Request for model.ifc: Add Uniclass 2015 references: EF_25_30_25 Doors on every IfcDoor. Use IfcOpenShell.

First a look at what the model holds.

```python
import ifcopenshell

model = ifcopenshell.open("model.ifc")
print(model.schema)
print("classifications:", [c.Name for c in model.by_type("IfcClassification")])
for ifc_class in ("IfcDoor", "IfcRoof", "IfcStair", "IfcWall", "IfcWindow"):
    print(ifc_class, len(model.by_type(ifc_class)))
```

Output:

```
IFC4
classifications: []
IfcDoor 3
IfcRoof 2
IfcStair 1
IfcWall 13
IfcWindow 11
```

```python
import ifcopenshell
import ifcopenshell.api.classification

model = ifcopenshell.open("model.ifc")

system = ifcopenshell.api.classification.add_classification(model, classification="Uniclass 2015")

codes = {
    "IfcDoor": ("EF_25_30_25", "Doors"),
}
for ifc_class, (code, name) in codes.items():
    products = model.by_type(ifc_class)
    ifcopenshell.api.classification.add_reference(
        model, products=products, classification=system, identification=code, name=name
    )
    print(code, len(products))

model.write("model_rev.ifc")
```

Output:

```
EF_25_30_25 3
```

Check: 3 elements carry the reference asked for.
